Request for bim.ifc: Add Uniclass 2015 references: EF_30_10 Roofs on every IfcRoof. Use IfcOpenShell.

First a look at what the model holds.

```python
import ifcopenshell

model = ifcopenshell.open("bim.ifc")
print(model.schema)
print("classifications:", [c.Name for c in model.by_type("IfcClassification")])
for ifc_class in ("IfcDoor", "IfcRoof", "IfcStair", "IfcWall", "IfcWindow"):
    print(ifc_class, len(model.by_type(ifc_class)))
```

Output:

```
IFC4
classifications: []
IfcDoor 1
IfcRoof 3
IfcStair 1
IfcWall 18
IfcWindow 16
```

```python
import ifcopenshell
import ifcopenshell.api.classification

model = ifcopenshell.open("bim.ifc")

system = ifcopenshell.api.classification.add_classification(model, classification="Uniclass 2015")

codes = {
    "IfcRoof": ("EF_30_10", "Roofs"),
}
for ifc_class, (code, name) in codes.items():
    products = model.by_type(ifc_class)
    ifcopenshell.api.classification.add_reference(
        model, products=products, classification=system, identification=code, name=name
    )
    print(code, len(products))

model.write("bim_v2.ifc")
```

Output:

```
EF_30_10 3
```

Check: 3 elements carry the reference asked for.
